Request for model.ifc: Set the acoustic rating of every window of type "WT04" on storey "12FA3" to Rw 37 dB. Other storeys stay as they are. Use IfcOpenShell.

First a look at what the model holds.

```python
import ifcopenshell
import ifcopenshell.util.element

model = ifcopenshell.open("model.ifc")
print(model.schema)
storey = next(s for s in model.by_type("IfcBuildingStorey") if s.Name == "12FA3")
windows = [e for e in ifcopenshell.util.element.get_decomposition(storey) if e.is_a("IfcWindow")]
seen = {}
for e in windows:
    element_type = ifcopenshell.util.element.get_type(e)
    key = (element_type.Name if element_type != e and element_type else None, ifcopenshell.util.element.get_pset(e, "Pset_WindowCommon", "AcousticRating"))
    seen[key] = seen.get(key, 0) + 1
for (name, value), count in sorted(seen.items(), key=str):
    print(count, "x", name, "|", value)
```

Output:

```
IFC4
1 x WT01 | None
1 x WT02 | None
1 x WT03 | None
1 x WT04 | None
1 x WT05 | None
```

```python
import ifcopenshell
import ifcopenshell.api.pset
import ifcopenshell.util.element

model = ifcopenshell.open("model.ifc")

storey = next(s for s in model.by_type("IfcBuildingStorey") if s.Name == "12FA3")
windows = [e for e in ifcopenshell.util.element.get_decomposition(storey) if e.is_a("IfcWindow")]

count = 0
for e in windows:
    element_type = ifcopenshell.util.element.get_type(e)
    if element_type in (None, e) or element_type.Name != "WT04":
        continue
    # add_pset returns the element's existing set when there is one.
    pset = ifcopenshell.api.pset.add_pset(model, product=e, name="Pset_WindowCommon")
    ifcopenshell.api.pset.edit_pset(model, pset=pset, properties={"AcousticRating": "Rw 37 dB"})
    count += 1

print(count, "windows updated")

model.write("model_rev.ifc")
```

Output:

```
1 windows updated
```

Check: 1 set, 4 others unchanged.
